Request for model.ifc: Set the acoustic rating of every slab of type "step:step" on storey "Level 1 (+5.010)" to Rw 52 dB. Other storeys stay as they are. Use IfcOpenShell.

First a look at what the model holds.

```python
import ifcopenshell
import ifcopenshell.util.element

model = ifcopenshell.open("model.ifc")
print(model.schema)
storey = next(s for s in model.by_type("IfcBuildingStorey") if s.Name == "Level 1 (+5.010)")
slabs = [e for e in ifcopenshell.util.element.get_decomposition(storey) if e.is_a("IfcSlab")]
seen = {}
for e in slabs:
    element_type = ifcopenshell.util.element.get_type(e)
    key = (element_type.Name if element_type != e and element_type else None, ifcopenshell.util.element.get_pset(e, "Pset_SlabCommon", "AcousticRating"))
    seen[key] = seen.get(key, 0) + 1
for (name, value), count in sorted(seen.items(), key=str):
    print(count, "x", name, "|", value)
```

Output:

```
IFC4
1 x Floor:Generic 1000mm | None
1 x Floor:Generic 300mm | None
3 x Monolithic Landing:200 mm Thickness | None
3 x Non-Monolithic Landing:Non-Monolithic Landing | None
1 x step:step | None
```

```python
import ifcopenshell
import ifcopenshell.api.pset
import ifcopenshell.util.element

model = ifcopenshell.open("model.ifc")

storey = next(s for s in model.by_type("IfcBuildingStorey") if s.Name == "Level 1 (+5.010)")
slabs = [e for e in ifcopenshell.util.element.get_decomposition(storey) if e.is_a("IfcSlab")]

count = 0
for e in slabs:
    element_type = ifcopenshell.util.element.get_type(e)
    if element_type in (None, e) or element_type.Name != "step:step":
        continue
    # add_pset returns the element's existing set when there is one.
    pset = ifcopenshell.api.pset.add_pset(model, product=e, name="Pset_SlabCommon")
    ifcopenshell.api.pset.edit_pset(model, pset=pset, properties={"AcousticRating": "Rw 52 dB"})
    count += 1

print(count, "slabs updated")

model.write("model_updated.ifc")
```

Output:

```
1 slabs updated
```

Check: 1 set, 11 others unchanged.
